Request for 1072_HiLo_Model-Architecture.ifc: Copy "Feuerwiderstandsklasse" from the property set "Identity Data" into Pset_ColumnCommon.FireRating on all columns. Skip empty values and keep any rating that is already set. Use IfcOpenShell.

First a look at what the model holds.

```python
import ifcopenshell
import ifcopenshell.util.element

model = ifcopenshell.open("1072_HiLo_Model-Architecture.ifc")
print(model.schema)
columns = model.by_type("IfcColumn")
print(len(columns), "columns")
for e in columns[:8]:
    source = ifcopenshell.util.element.get_pset(e, "Identity Data", "Feuerwiderstandsklasse")
    target = ifcopenshell.util.element.get_pset(e, "Pset_ColumnCommon", "FireRating")
    print(e.id(), repr(source), repr(target), sep=" | ")
```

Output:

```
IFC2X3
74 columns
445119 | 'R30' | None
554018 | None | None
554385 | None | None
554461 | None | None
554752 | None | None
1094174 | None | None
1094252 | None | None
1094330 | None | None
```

```python
import ifcopenshell
import ifcopenshell.api.pset
import ifcopenshell.util.element

model = ifcopenshell.open("1072_HiLo_Model-Architecture.ifc")

count = 0
for e in model.by_type("IfcColumn"):
    value = ifcopenshell.util.element.get_pset(e, "Identity Data", "Feuerwiderstandsklasse")
    current = ifcopenshell.util.element.get_pset(e, "Pset_ColumnCommon", "FireRating")
    if not value or not value.strip() or current:
        continue
    # add_pset returns the element's existing set when there is one.
    pset = ifcopenshell.api.pset.add_pset(model, product=e, name="Pset_ColumnCommon")
    ifcopenshell.api.pset.edit_pset(model, pset=pset, properties={"FireRating": value})
    count += 1

print(count, "columns updated")

model.write("1072_HiLo_Model-Architecture_v2.ifc")
```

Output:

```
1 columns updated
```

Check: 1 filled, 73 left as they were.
